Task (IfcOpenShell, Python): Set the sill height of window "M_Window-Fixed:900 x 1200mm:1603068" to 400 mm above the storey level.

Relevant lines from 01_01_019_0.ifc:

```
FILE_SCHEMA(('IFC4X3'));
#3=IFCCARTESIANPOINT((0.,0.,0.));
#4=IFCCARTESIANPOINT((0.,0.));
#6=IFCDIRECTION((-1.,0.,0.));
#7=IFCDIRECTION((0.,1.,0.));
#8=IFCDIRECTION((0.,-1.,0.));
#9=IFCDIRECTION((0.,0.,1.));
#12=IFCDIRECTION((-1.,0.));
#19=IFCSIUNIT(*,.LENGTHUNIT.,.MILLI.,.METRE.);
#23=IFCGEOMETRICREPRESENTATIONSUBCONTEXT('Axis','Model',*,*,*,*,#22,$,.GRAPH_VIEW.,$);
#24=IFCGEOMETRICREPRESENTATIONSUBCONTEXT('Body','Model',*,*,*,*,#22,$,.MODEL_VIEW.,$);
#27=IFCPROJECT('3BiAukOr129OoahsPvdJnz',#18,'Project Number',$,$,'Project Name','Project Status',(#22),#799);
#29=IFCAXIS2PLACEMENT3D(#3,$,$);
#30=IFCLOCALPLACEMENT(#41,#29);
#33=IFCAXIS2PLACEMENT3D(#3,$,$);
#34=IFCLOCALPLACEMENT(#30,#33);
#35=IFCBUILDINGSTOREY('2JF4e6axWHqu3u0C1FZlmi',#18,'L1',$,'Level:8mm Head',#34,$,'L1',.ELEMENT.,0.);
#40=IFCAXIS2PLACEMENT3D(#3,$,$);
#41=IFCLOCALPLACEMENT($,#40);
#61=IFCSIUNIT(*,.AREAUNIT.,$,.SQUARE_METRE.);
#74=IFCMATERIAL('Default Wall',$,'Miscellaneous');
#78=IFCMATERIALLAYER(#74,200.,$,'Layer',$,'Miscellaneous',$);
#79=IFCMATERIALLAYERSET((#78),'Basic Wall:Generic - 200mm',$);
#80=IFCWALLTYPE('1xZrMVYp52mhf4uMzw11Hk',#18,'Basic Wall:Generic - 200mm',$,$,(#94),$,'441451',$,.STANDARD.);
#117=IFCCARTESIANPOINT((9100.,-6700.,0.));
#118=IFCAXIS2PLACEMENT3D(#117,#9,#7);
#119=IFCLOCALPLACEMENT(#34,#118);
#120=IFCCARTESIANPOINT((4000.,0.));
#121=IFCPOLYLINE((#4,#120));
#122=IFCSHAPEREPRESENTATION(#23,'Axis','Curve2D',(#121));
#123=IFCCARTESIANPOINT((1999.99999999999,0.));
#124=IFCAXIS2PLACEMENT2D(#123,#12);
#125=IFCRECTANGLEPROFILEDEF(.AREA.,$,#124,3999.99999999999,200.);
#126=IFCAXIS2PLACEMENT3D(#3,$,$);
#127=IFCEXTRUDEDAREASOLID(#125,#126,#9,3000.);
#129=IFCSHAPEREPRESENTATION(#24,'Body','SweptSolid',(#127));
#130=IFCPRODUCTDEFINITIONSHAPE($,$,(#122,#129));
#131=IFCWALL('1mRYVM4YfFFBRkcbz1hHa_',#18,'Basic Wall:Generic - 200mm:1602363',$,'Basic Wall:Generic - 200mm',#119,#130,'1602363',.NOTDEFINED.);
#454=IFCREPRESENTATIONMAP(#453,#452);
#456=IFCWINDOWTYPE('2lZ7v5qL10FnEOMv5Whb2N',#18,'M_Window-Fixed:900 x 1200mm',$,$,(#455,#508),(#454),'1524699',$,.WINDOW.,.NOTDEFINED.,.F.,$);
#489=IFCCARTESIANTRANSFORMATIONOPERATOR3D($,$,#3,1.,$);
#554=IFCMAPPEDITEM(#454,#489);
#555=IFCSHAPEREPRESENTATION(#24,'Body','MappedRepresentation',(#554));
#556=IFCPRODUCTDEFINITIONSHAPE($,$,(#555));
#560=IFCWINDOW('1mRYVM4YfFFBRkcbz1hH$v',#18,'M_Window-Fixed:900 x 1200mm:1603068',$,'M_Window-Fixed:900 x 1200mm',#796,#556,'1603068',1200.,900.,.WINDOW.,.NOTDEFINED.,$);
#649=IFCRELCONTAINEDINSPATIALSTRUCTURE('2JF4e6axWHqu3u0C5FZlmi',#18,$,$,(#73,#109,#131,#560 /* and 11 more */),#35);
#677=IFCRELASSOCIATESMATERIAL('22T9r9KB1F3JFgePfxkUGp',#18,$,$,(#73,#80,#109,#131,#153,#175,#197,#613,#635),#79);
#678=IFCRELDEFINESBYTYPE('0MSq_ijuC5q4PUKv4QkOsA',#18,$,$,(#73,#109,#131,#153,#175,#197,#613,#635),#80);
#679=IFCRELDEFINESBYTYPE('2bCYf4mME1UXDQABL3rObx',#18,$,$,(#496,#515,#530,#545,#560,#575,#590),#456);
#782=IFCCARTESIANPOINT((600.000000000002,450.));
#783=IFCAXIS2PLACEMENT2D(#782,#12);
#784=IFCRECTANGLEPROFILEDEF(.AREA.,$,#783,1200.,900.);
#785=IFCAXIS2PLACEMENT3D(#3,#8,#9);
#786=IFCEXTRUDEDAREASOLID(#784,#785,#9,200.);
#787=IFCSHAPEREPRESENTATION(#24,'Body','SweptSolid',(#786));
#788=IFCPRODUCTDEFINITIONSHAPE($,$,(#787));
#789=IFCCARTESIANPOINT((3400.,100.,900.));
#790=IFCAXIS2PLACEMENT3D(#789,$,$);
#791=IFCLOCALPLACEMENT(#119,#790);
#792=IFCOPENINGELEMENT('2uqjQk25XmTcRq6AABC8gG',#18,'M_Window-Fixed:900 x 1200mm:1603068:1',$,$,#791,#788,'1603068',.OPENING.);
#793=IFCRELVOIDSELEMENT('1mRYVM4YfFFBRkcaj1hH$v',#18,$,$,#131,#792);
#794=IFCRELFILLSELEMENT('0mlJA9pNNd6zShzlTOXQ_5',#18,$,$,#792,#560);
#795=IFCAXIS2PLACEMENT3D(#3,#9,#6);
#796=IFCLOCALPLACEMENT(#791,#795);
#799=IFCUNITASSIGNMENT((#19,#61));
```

```python
import numpy as np
import ifcopenshell
import ifcopenshell.api.geometry
import ifcopenshell.geom
import ifcopenshell.util.element
import ifcopenshell.util.placement
import ifcopenshell.util.shape
import ifcopenshell.util.unit

model = ifcopenshell.open("01_01_019_0.ifc")
unit_scale = ifcopenshell.util.unit.calculate_unit_scale(model)

window = model.by_guid("1mRYVM4YfFFBRkcbz1hH$v")
opening = window.FillsVoids[0].RelatingOpeningElement
storey = ifcopenshell.util.element.get_container(window, ifc_class="IfcBuildingStorey")
level = ifcopenshell.util.placement.get_local_placement(storey.ObjectPlacement)[2, 3]

# The opening's origin need not be at the sill, so measure its lowest point.
shape = ifcopenshell.geom.create_shape(ifcopenshell.geom.settings(), opening)
bottom = ifcopenshell.util.shape.get_shape_bottom_elevation(shape, shape.geometry) / unit_scale
dz = level + 0.4 / unit_scale - bottom

shift = np.array([0.0, 0.0, dz])
# The window is placed relative to its opening, so it follows when the opening moves.
matrix = ifcopenshell.util.placement.get_local_placement(opening.ObjectPlacement)
matrix[:3, 3] += shift
ifcopenshell.api.geometry.edit_object_placement(
    model, product=opening, matrix=matrix, is_si=False, should_transform_children=True
)

print(f"moved by {dz * unit_scale:+.3f} m")

model.write("01_01_019_0_v2.ifc")
```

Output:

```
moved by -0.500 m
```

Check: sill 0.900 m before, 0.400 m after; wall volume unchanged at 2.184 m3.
